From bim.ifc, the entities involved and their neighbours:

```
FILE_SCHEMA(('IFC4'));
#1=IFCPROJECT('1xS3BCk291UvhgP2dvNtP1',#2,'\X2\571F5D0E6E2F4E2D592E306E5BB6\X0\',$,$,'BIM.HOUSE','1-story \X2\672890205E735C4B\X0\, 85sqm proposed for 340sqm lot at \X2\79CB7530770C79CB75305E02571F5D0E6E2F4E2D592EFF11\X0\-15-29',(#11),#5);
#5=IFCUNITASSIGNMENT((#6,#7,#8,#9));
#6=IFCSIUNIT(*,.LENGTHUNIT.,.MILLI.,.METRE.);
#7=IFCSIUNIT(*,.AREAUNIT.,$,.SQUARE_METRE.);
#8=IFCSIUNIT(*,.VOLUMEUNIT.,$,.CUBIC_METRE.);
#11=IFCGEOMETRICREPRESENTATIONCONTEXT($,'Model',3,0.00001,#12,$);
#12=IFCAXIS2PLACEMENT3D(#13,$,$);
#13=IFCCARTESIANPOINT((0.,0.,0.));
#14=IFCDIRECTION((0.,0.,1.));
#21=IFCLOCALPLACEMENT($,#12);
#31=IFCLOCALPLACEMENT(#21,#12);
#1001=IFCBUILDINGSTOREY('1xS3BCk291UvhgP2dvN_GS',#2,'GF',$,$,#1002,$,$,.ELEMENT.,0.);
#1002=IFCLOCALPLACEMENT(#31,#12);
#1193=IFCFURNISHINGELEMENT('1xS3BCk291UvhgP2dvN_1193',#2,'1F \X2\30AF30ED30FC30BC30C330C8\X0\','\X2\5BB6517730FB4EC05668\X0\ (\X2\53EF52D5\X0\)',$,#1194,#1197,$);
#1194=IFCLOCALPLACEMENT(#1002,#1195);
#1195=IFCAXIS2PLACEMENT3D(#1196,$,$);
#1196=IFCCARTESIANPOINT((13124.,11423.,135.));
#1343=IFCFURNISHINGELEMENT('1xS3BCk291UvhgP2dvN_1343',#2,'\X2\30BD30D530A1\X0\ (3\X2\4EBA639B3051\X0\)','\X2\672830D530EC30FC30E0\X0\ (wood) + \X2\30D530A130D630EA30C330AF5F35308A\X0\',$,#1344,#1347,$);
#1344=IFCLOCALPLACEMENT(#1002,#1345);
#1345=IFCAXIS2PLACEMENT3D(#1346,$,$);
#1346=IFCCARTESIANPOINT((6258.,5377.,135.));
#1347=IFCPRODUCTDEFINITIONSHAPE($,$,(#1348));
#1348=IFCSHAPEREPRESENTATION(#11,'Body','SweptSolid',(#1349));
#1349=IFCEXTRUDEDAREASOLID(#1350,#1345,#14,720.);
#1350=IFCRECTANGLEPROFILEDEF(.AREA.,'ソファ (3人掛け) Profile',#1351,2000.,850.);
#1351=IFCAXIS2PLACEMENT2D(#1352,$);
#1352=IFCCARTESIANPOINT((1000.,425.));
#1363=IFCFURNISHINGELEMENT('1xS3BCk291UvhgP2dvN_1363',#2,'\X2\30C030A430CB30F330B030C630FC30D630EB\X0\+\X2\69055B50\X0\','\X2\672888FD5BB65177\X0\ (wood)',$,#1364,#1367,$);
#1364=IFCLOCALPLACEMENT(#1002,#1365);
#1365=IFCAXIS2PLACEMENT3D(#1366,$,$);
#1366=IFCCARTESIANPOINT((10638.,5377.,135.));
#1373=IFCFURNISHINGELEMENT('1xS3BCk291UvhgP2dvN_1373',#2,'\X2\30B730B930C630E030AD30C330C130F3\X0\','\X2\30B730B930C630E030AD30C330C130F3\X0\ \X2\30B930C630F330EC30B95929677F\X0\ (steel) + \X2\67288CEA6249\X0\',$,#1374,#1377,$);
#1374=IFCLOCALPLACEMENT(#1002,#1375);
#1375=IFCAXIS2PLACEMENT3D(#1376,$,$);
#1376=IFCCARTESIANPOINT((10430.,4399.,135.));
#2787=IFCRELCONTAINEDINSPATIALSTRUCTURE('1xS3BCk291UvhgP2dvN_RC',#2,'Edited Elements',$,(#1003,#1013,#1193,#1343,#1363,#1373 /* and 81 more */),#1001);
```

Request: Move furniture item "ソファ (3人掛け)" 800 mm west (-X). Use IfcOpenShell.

```python
import ifcopenshell
import ifcopenshell.api.geometry
import ifcopenshell.util.placement
import ifcopenshell.util.unit

model = ifcopenshell.open("bim.ifc")
unit_scale = ifcopenshell.util.unit.calculate_unit_scale(model)

item = model.by_guid("1xS3BCk291UvhgP2dvN_1343")
matrix = ifcopenshell.util.placement.get_local_placement(item.ObjectPlacement)
matrix[0, 3] -= 0.8 / unit_scale
ifcopenshell.api.geometry.edit_object_placement(model, product=item, matrix=matrix, is_si=False)

print(ifcopenshell.util.placement.get_local_placement(item.ObjectPlacement).round(3) + 0.0)

model.write("bim_v2.ifc")
```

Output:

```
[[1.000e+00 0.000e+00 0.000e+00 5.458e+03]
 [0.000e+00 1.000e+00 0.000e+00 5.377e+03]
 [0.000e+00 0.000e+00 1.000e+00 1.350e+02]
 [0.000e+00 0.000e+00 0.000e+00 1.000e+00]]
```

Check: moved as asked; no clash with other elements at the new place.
